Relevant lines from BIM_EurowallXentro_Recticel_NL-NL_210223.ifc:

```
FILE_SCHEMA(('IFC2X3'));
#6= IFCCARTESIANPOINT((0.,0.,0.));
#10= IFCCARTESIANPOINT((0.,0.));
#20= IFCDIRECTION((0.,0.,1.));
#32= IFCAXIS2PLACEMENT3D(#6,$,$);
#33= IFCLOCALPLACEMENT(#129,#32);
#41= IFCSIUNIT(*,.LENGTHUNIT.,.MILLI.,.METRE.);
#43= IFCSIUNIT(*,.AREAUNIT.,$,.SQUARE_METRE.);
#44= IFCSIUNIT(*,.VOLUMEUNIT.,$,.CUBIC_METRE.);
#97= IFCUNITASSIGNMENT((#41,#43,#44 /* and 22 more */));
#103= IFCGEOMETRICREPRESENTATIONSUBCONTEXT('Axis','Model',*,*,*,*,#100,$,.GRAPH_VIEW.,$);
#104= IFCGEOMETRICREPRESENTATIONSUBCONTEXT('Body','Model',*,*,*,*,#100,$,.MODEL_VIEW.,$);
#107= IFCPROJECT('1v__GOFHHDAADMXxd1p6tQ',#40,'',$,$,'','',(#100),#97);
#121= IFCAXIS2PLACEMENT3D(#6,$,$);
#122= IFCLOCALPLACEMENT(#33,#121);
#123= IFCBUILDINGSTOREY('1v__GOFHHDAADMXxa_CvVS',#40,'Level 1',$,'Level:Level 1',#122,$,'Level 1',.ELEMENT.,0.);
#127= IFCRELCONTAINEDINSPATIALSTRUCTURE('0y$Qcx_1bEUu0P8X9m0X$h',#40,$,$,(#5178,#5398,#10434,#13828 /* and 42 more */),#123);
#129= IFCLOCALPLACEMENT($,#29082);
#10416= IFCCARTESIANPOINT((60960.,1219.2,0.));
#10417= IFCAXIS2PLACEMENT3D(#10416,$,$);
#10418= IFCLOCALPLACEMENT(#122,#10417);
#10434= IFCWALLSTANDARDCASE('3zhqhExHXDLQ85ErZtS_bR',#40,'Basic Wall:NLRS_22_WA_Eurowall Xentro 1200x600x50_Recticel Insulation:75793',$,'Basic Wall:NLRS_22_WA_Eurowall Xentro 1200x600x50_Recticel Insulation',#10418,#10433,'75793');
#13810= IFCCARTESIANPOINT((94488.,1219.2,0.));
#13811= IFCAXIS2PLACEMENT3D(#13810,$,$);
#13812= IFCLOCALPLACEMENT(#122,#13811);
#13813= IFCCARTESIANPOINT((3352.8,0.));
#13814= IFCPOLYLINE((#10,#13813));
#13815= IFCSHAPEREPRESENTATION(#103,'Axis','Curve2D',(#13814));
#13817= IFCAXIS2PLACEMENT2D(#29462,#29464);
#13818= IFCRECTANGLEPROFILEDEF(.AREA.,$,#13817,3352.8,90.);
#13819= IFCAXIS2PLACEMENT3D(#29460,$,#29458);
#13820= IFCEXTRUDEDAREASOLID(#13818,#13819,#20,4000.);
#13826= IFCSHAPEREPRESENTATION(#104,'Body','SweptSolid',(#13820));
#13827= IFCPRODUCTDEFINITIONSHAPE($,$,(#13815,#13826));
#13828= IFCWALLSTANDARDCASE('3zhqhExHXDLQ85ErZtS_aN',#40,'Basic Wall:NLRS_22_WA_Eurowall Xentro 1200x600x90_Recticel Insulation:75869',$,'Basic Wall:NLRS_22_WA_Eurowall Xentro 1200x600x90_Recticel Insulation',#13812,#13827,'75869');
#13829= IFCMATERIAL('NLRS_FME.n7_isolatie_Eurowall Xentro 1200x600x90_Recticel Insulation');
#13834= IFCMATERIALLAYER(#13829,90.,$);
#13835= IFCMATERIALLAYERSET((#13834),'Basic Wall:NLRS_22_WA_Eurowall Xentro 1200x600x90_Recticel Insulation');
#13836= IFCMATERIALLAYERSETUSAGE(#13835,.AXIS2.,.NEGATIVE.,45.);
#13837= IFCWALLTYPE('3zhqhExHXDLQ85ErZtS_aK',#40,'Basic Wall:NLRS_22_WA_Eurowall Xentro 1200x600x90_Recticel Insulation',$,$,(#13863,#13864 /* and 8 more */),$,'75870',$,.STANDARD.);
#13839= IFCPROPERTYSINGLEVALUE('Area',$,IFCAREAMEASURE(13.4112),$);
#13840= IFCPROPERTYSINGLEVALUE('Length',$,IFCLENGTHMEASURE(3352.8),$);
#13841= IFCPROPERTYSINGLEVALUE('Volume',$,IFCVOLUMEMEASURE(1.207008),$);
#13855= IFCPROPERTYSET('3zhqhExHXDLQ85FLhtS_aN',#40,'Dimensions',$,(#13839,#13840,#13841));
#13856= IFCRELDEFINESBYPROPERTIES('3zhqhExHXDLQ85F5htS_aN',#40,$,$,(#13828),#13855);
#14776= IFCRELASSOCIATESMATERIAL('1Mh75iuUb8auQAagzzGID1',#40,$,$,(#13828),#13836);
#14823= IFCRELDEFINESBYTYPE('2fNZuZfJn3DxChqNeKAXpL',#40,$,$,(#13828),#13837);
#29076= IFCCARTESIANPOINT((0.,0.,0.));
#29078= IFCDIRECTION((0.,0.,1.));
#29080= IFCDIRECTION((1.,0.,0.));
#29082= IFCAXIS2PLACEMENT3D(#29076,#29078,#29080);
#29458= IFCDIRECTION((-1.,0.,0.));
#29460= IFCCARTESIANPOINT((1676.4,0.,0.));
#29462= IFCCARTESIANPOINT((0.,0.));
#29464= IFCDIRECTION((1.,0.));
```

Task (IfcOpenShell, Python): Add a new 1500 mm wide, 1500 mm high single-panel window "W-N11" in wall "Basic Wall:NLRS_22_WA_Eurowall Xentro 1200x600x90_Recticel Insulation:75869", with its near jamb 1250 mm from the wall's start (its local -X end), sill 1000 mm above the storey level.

```python
import numpy as np
import ifcopenshell
import ifcopenshell.api.feature
import ifcopenshell.api.geometry
import ifcopenshell.api.pset
import ifcopenshell.api.root
import ifcopenshell.api.spatial
import ifcopenshell.api.type
import ifcopenshell.geom
import ifcopenshell.util.element
import ifcopenshell.util.placement
import ifcopenshell.util.representation
import ifcopenshell.util.shape
import ifcopenshell.util.unit

model = ifcopenshell.open("BIM_EurowallXentro_Recticel_NL-NL_210223.ifc")
unit_scale = ifcopenshell.util.unit.calculate_unit_scale(model)
area_scale = ifcopenshell.util.unit.calculate_unit_scale(model, "AREAUNIT")
volume_scale = ifcopenshell.util.unit.calculate_unit_scale(model, "VOLUMEUNIT")
settings = ifcopenshell.geom.settings()


def volume(element):
    """Net volume in cubic metres, openings subtracted."""
    shape = ifcopenshell.geom.create_shape(settings, element)
    return ifcopenshell.util.shape.get_volume(shape.geometry)


wall = model.by_guid("3zhqhExHXDLQ85ErZtS_aN")
storey = ifcopenshell.util.element.get_container(wall, ifc_class="IfcBuildingStorey")
context = ifcopenshell.util.representation.get_context(model, "Model", "Body", "MODEL_VIEW")
before = volume(wall)

width, height, from_end, sill = 1.5, 1.5, 1.25, 1  # metres

# The wall runs along its own X axis, and the end named is its -X end.
wall_shape = ifcopenshell.geom.create_shape(settings, wall)
x, y, z = ifcopenshell.util.shape.get_vertices(wall_shape.geometry).T
start = x.min() + from_end
face, thickness = float(y.min()), float(y.max() - y.min())
wall_matrix = ifcopenshell.util.placement.get_local_placement(wall.ObjectPlacement)
level = ifcopenshell.util.placement.get_local_placement(storey.ObjectPlacement)[2, 3]


def in_wall(x, y):
    """Placement at x, y metres in the wall's axes, at sill height."""
    matrix = wall_matrix.copy()
    matrix[:, 3] = wall_matrix @ np.array([x / unit_scale, y / unit_scale, 0.0, 1.0])
    matrix[2, 3] = level + sill / unit_scale
    return matrix


# Opening: a box that overshoots both wall faces by 50 mm.
opening = ifcopenshell.api.root.create_entity(model, ifc_class="IfcOpeningElement")
box = ifcopenshell.api.geometry.add_wall_representation(
    model, context=context, length=width, height=height, thickness=thickness + 0.1
)
ifcopenshell.api.geometry.assign_representation(model, product=opening, representation=box)
ifcopenshell.api.geometry.edit_object_placement(model, product=opening, matrix=in_wall(start, face - 0.05), is_si=False)
ifcopenshell.api.feature.add_feature(model, feature=opening, element=wall)

window = ifcopenshell.api.root.create_entity(model, ifc_class="IfcWindow", name="W-N11")
window.OverallWidth, window.OverallHeight = width / unit_scale, height / unit_scale
body = ifcopenshell.api.geometry.add_window_representation(
    model,
    context=context,
    overall_width=window.OverallWidth,
    overall_height=window.OverallHeight,
    partition_type="SINGLE_PANEL",
)
ifcopenshell.api.geometry.assign_representation(model, product=window, representation=body)
ifcopenshell.api.spatial.assign_container(model, products=[window], relating_structure=storey)
fills = ifcopenshell.api.feature.add_filling(model, opening=opening, element=window)
fills.OwnerHistory = window.OwnerHistory  # required in IFC2X3

# IFC2X3 keeps the operation on the window style.
style = ifcopenshell.api.root.create_entity(model, ifc_class="IfcWindowStyle", name="W-N11")
style.OperationType, style.ConstructionType = "SINGLE_PANEL", "NOTDEFINED"
style.ParameterTakesPrecedence = style.Sizeable = False
ifcopenshell.api.type.assign_type(model, related_objects=[window], relating_type=style)

# Centre the window in the wall's thickness.
ifcopenshell.api.geometry.edit_object_placement(model, product=window, matrix=in_wall(start, face), is_si=False)
window_shape = ifcopenshell.geom.create_shape(settings, window)
depth = ifcopenshell.util.shape.get_vertices(window_shape.geometry)[:, 1]
offset = face + thickness / 2 - (depth.min() + depth.max()) / 2
ifcopenshell.api.geometry.edit_object_placement(model, product=window, matrix=in_wall(start, offset), is_si=False)

after = volume(wall)

# Update the wall's stored quantities.
pset = model.by_id(ifcopenshell.util.element.get_pset(wall, "Dimensions", should_inherit=False)["id"])
ifcopenshell.api.pset.edit_pset(model, pset=pset, properties={
    "Area": model.create_entity("IfcAreaMeasure", after / thickness / area_scale),
    "Volume": model.create_entity("IfcVolumeMeasure", after / volume_scale),
})

print(f"wall volume {before:.3f} -> {after:.3f} m3")

model.write("BIM_EurowallXentro_Recticel_NL-NL_210223_updated.ifc")
```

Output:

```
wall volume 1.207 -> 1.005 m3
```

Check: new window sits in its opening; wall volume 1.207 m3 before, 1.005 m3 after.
